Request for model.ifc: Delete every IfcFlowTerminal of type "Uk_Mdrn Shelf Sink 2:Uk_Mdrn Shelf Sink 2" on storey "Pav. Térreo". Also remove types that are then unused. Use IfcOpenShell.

First a look at what the model holds.

```python
import ifcopenshell
import ifcopenshell.util.element

model = ifcopenshell.open("model.ifc")
print(model.schema)
storey = next(s for s in model.by_type("IfcBuildingStorey") if s.Name == "Pav. Térreo")
terminals = [e for e in ifcopenshell.util.element.get_decomposition(storey) if e.is_a("IfcFlowTerminal")]
seen = {}
for e in terminals:
    element_type = ifcopenshell.util.element.get_type(e)
    name = element_type.Name if element_type not in (None, e) else None
    seen[name] = seen.get(name, 0) + 1
for name, count in sorted(seen.items(), key=str):
    print(count, "x", name)
```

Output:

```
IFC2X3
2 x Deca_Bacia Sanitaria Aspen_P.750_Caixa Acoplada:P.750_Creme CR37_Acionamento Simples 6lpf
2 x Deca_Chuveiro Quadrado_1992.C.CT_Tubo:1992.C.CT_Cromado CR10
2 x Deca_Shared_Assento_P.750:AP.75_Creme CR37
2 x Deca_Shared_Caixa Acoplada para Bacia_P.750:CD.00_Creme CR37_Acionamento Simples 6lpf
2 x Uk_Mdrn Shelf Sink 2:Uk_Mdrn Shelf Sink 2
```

```python
import ifcopenshell
import ifcopenshell.api.root
import ifcopenshell.util.element

model = ifcopenshell.open("model.ifc")

storey = next(s for s in model.by_type("IfcBuildingStorey") if s.Name == "Pav. Térreo")
terminals = [e for e in ifcopenshell.util.element.get_decomposition(storey) if e.is_a("IfcFlowTerminal")]
targets = [e for e in terminals if (t := ifcopenshell.util.element.get_type(e)) not in (None, e) and t.Name == "Uk_Mdrn Shelf Sink 2:Uk_Mdrn Shelf Sink 2"]
types = {ifcopenshell.util.element.get_type(e) for e in targets} - {None, *targets}

for e in targets:
    ifcopenshell.api.root.remove_product(model, product=e)
print(len(targets), "removed")

unused = [t for t in types if not ifcopenshell.util.element.get_types(t)]
for t in unused:
    ifcopenshell.api.root.remove_product(model, product=t)
print(len(unused), "unused types removed")

model.write("model_updated.ifc")
```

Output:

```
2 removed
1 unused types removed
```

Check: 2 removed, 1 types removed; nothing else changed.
